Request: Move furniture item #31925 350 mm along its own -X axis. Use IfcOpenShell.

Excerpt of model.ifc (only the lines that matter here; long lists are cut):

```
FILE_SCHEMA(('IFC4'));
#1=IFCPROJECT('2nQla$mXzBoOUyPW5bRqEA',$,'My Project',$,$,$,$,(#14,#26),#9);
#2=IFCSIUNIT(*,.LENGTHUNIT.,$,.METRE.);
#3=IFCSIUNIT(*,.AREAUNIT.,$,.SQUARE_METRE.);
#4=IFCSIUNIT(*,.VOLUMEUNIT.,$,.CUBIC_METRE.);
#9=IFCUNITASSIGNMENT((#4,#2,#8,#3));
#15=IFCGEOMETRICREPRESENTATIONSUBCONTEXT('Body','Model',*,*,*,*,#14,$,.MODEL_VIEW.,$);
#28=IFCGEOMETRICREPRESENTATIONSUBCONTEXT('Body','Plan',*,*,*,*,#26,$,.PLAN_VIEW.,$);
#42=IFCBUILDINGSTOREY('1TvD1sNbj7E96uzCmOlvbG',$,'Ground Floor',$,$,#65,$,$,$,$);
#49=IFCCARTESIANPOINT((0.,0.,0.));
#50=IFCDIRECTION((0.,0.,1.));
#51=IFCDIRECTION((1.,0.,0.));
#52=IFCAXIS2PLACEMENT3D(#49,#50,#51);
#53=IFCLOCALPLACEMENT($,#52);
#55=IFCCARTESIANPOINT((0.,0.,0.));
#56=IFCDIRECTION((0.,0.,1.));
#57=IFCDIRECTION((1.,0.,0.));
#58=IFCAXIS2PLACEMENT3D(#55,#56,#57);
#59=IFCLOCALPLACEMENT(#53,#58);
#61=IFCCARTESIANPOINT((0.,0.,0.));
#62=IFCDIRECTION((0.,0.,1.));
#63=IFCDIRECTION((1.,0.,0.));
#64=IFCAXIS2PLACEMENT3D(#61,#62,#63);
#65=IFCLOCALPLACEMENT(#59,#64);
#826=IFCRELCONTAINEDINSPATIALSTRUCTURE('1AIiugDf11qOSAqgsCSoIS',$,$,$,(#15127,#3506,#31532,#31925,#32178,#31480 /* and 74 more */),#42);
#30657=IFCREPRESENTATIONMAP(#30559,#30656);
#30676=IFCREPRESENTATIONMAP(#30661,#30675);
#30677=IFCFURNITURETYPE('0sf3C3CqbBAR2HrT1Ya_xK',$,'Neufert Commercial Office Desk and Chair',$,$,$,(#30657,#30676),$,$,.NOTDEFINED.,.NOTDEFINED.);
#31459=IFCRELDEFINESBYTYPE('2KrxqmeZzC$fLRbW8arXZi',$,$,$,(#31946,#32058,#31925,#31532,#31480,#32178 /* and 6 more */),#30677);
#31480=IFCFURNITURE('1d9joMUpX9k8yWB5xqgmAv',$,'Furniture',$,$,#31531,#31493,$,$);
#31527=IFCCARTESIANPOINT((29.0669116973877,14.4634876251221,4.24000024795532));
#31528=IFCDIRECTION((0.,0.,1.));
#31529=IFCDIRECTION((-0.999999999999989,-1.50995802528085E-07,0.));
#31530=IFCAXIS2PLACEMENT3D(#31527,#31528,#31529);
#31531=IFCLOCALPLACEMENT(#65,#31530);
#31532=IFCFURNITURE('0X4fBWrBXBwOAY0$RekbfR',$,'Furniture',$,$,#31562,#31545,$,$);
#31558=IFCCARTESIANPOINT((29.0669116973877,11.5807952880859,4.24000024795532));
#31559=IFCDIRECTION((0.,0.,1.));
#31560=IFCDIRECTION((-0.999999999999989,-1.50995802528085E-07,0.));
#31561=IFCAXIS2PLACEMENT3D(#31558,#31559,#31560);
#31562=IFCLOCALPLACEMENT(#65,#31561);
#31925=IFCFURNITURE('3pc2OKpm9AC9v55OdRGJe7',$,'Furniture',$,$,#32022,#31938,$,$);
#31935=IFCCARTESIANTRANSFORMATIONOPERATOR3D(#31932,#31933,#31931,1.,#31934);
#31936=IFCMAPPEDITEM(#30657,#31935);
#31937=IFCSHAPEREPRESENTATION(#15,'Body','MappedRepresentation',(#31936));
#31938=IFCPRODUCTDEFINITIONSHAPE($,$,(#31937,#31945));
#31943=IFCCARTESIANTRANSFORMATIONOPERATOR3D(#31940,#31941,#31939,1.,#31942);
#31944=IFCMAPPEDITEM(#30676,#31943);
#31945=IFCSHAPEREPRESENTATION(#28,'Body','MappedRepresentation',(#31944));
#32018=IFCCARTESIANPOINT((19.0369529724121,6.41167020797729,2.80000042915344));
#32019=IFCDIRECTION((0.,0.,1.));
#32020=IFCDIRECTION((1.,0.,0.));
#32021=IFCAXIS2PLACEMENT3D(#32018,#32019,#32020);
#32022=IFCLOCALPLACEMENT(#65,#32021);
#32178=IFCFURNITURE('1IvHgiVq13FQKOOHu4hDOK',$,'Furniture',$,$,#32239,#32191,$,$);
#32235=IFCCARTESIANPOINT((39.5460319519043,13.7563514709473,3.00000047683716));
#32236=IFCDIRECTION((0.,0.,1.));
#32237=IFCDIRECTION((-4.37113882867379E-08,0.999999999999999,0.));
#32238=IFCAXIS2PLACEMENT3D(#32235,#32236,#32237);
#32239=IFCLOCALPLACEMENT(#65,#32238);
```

```python
import ifcopenshell
import ifcopenshell.api.geometry
import ifcopenshell.util.placement

model = ifcopenshell.open("model.ifc")

item = model.by_id(31925)
matrix = ifcopenshell.util.placement.get_local_placement(item.ObjectPlacement)
matrix[:3, 3] -= matrix[:3, 0] * 0.35
ifcopenshell.api.geometry.edit_object_placement(model, product=item, matrix=matrix, is_si=False)

print(ifcopenshell.util.placement.get_local_placement(item.ObjectPlacement).round(3) + 0.0)

model.write("model-out.ifc")
```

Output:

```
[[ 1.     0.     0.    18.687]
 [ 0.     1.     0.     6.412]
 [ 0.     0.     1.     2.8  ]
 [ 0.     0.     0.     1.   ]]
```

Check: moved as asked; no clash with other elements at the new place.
